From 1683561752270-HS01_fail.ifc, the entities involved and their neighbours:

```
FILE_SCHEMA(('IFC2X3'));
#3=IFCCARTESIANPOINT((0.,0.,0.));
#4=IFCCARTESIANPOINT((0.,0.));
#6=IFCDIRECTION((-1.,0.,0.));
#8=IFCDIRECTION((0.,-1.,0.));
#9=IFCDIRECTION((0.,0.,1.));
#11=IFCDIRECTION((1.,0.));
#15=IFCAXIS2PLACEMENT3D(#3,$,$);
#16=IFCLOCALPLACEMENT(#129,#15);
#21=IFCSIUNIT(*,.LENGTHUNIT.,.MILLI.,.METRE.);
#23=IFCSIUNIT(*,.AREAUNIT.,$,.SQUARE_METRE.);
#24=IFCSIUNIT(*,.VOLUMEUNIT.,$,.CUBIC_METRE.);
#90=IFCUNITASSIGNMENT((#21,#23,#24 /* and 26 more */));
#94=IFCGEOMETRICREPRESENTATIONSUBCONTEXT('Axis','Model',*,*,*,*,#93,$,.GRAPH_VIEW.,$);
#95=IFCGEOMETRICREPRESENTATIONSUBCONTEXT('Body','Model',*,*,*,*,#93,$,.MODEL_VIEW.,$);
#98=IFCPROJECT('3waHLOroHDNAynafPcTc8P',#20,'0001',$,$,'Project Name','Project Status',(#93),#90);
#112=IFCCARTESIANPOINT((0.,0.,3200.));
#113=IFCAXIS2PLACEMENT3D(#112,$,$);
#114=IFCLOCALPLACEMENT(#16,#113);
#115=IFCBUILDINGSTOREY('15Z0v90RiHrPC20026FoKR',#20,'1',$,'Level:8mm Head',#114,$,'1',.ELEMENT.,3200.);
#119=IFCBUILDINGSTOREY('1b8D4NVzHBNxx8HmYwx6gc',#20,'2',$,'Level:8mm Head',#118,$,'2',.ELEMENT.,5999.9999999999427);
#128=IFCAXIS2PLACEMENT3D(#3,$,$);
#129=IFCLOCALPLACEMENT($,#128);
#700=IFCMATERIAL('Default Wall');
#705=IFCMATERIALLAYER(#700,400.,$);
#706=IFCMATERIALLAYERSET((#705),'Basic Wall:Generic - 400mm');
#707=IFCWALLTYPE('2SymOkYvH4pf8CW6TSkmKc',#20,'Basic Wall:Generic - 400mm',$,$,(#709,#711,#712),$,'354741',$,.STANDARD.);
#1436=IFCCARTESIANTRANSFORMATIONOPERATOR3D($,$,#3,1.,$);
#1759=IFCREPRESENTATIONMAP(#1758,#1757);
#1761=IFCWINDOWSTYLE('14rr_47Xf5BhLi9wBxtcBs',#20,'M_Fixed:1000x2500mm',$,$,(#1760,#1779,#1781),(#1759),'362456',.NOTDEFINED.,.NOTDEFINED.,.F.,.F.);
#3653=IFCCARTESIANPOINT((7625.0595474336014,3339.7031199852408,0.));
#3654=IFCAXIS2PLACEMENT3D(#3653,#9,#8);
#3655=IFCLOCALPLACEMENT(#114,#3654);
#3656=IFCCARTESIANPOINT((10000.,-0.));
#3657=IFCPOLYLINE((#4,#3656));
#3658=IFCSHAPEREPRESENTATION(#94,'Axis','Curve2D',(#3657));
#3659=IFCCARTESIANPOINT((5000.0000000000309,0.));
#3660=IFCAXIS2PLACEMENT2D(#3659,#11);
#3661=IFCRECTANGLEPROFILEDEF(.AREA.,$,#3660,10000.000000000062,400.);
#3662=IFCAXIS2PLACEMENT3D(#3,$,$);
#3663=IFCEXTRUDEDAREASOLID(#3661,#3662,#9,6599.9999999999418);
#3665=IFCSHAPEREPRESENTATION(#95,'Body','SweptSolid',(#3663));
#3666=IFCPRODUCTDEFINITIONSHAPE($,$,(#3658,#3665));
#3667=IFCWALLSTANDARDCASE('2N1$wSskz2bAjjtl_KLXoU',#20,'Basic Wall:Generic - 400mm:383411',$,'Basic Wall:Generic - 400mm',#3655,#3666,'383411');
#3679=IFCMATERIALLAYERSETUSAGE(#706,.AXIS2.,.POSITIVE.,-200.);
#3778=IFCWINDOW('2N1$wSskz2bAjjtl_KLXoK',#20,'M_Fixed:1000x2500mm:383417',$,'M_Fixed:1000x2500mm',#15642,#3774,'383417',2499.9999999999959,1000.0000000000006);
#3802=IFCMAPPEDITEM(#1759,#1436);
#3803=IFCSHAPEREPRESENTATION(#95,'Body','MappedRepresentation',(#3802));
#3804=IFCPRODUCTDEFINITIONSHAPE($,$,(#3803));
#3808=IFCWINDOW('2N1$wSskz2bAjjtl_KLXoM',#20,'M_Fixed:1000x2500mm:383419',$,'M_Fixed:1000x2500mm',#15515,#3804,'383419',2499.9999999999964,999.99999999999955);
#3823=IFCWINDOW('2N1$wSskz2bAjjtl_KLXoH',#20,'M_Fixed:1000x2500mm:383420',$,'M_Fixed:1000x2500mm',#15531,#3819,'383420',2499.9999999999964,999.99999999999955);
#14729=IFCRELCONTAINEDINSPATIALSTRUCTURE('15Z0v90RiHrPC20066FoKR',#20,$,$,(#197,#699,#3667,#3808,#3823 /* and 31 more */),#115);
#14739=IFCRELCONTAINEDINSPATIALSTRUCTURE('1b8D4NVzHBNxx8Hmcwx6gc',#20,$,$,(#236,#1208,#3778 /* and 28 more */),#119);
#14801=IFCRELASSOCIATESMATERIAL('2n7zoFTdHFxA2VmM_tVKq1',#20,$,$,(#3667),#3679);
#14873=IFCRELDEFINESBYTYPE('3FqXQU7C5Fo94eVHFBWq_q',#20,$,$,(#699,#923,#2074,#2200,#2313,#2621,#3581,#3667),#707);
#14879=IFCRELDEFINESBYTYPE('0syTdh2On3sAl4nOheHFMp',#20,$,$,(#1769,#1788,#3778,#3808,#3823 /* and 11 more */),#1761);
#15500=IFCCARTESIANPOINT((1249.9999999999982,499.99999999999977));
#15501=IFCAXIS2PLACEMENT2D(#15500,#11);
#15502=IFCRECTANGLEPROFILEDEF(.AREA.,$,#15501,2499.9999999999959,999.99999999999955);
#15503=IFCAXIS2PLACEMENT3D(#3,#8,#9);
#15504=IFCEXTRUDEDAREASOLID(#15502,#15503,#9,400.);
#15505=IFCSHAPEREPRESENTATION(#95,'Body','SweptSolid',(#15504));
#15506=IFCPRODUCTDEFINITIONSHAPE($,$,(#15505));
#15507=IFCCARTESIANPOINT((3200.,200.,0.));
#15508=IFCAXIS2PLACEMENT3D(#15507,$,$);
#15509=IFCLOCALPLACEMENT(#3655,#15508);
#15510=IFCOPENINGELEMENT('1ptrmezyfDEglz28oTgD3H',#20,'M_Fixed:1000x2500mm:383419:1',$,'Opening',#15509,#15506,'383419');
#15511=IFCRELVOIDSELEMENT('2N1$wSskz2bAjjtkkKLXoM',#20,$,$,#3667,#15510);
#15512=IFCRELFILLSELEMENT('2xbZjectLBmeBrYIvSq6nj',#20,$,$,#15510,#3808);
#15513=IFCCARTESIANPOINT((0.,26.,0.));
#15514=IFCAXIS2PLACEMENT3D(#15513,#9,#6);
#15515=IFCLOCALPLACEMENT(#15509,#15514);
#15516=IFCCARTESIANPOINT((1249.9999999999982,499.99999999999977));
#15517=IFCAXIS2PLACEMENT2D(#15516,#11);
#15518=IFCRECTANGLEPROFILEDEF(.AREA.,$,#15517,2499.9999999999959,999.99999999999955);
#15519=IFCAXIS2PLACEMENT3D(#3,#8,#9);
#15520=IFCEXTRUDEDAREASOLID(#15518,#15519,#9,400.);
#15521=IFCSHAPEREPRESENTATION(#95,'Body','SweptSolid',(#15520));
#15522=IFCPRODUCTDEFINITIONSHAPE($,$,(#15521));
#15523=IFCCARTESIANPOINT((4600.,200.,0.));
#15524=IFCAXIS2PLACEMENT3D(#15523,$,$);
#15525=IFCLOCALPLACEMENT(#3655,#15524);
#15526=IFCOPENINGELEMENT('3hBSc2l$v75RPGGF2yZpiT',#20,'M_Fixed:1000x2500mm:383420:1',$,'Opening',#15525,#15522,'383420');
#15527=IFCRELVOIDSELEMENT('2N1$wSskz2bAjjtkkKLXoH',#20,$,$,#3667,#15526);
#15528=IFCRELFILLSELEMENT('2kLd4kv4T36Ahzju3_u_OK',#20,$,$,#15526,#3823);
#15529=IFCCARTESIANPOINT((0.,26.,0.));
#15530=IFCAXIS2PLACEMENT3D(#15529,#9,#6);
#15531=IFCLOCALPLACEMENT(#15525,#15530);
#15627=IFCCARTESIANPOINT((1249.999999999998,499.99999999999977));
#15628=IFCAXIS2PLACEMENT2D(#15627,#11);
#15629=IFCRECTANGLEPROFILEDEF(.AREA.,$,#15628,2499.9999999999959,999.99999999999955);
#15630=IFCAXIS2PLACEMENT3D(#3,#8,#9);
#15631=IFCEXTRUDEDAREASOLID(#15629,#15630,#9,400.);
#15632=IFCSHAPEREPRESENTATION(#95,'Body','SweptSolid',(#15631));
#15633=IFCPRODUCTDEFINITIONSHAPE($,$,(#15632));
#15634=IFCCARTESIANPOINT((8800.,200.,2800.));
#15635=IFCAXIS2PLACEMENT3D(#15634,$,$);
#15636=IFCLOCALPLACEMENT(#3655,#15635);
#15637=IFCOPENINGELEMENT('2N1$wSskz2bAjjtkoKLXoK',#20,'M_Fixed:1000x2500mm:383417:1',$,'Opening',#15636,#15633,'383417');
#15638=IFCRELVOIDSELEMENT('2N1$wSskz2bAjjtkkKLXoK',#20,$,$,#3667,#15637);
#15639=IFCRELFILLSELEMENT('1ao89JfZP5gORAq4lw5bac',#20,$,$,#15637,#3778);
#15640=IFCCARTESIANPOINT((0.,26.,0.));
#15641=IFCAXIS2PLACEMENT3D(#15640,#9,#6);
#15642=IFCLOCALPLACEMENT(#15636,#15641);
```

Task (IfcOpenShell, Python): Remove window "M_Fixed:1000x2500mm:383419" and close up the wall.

```python
import ifcopenshell
import ifcopenshell.api.feature
import ifcopenshell.api.root
import ifcopenshell.geom
import ifcopenshell.util.shape

model = ifcopenshell.open("1683561752270-HS01_fail.ifc")
settings = ifcopenshell.geom.settings()


def volume(element):
    """Net volume in cubic metres, openings subtracted."""
    shape = ifcopenshell.geom.create_shape(settings, element)
    return ifcopenshell.util.shape.get_volume(shape.geometry)


window = model.by_guid("2N1$wSskz2bAjjtl_KLXoM")
opening = window.FillsVoids[0].RelatingOpeningElement
wall = opening.VoidsElements[0].RelatingBuildingElement
before = volume(wall)

ifcopenshell.api.root.remove_product(model, product=window)
ifcopenshell.api.feature.remove_feature(model, feature=opening)

after = volume(wall)

print(f"wall volume {before:.3f} -> {after:.3f} m3")

model.write("1683561752270-HS01_fail_v2.ifc")
```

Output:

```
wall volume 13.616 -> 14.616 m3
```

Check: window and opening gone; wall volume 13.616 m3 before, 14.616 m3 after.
